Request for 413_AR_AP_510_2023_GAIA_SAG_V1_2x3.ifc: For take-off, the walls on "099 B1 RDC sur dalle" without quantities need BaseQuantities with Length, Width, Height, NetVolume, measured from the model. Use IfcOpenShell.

First a look at what the model holds.

```python
import ifcopenshell
import ifcopenshell.util.element
import ifcopenshell.util.unit

model = ifcopenshell.open("413_AR_AP_510_2023_GAIA_SAG_V1_2x3.ifc")
print(model.schema)
for unit_type in ("LENGTHUNIT", "AREAUNIT", "VOLUMEUNIT"):
    print(unit_type, ifcopenshell.util.unit.calculate_unit_scale(model, unit_type))
storey = next(s for s in model.by_type("IfcBuildingStorey") if s.Name == "099 B1 RDC sur dalle")
walls = [e for e in ifcopenshell.util.element.get_decomposition(storey) if e.is_a("IfcWall")]
for e in sorted(walls, key=lambda e: e.id()):
    print(e.id(), e.is_a(), e.Name, list(ifcopenshell.util.element.get_psets(e, qtos_only=True)), sep=" | ")
```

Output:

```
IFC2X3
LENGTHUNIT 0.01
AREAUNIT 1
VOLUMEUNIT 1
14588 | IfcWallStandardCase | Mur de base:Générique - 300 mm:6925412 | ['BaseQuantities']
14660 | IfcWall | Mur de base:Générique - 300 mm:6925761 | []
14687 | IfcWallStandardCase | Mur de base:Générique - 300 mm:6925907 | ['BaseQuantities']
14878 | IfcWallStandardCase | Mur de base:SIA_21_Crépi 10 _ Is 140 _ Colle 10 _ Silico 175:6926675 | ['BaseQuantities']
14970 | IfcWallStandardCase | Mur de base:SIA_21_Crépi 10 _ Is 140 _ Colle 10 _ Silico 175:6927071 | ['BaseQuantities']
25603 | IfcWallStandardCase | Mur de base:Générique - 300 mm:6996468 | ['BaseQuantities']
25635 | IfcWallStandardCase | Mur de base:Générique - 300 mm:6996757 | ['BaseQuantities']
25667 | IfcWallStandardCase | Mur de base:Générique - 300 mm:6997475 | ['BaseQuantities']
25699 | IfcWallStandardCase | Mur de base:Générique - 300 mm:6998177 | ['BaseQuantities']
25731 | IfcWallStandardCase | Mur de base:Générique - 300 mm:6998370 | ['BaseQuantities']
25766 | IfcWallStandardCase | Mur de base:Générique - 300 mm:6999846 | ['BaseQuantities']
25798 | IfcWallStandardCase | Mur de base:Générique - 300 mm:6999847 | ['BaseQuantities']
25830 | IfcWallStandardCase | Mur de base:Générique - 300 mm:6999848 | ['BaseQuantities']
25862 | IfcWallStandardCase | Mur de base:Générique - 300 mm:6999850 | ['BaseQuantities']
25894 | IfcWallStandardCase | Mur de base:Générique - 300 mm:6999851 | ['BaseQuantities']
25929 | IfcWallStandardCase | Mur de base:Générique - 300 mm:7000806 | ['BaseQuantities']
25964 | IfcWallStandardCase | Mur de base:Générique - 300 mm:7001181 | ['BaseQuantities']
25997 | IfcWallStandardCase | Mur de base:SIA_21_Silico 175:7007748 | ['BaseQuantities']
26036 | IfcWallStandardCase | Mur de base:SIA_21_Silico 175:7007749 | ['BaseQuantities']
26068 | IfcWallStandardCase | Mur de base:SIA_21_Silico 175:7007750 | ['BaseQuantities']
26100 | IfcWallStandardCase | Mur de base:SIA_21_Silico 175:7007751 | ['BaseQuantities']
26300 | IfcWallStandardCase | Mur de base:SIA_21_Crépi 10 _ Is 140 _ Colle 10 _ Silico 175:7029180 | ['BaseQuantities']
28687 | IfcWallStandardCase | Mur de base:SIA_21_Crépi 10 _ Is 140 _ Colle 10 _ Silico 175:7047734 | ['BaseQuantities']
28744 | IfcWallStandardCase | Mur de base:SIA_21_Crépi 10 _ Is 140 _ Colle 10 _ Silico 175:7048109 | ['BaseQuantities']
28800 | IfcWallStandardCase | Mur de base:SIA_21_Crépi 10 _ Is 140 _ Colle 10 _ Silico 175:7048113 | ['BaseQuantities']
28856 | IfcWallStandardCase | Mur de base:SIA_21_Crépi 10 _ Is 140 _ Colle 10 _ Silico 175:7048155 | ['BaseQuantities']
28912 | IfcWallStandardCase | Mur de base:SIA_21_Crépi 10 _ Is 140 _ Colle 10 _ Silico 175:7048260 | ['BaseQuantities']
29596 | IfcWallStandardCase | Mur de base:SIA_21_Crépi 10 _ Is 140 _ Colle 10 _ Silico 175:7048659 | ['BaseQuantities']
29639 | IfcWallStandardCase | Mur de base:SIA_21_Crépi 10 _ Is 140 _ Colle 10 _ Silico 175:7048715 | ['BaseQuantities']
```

```python
import ifcopenshell
import ifcopenshell.api.pset
import ifcopenshell.geom
import ifcopenshell.util.element
import ifcopenshell.util.shape
import ifcopenshell.util.unit

model = ifcopenshell.open("413_AR_AP_510_2023_GAIA_SAG_V1_2x3.ifc")
unit_scale = ifcopenshell.util.unit.calculate_unit_scale(model)
volume_scale = ifcopenshell.util.unit.calculate_unit_scale(model, "VOLUMEUNIT")
settings = ifcopenshell.geom.settings()

storey = next(s for s in model.by_type("IfcBuildingStorey") if s.Name == "099 B1 RDC sur dalle")
walls = [e for e in ifcopenshell.util.element.get_decomposition(storey) if e.is_a("IfcWall")]

for e in sorted(walls, key=lambda e: e.id()):
    if ifcopenshell.util.element.get_psets(e, qtos_only=True, should_inherit=False):
        continue
    # Geometry comes back in metres, in the element's own axes.
    shape = ifcopenshell.geom.create_shape(settings, e)
    values = {
        "Length": ifcopenshell.util.shape.get_x(shape.geometry) / unit_scale,
        "Width": ifcopenshell.util.shape.get_y(shape.geometry) / unit_scale,
        "Height": ifcopenshell.util.shape.get_z(shape.geometry) / unit_scale,
        "NetVolume": ifcopenshell.util.shape.get_volume(shape.geometry) / volume_scale,
    }
    qto = ifcopenshell.api.pset.add_qto(model, product=e, name="BaseQuantities")
    ifcopenshell.api.pset.edit_qto(model, qto=qto, properties=values)
    print(e.id(), {k: round(v, 3) for k, v in values.items()})

model.write("413_AR_AP_510_2023_GAIA_SAG_V1_2x3_rev.ifc")
```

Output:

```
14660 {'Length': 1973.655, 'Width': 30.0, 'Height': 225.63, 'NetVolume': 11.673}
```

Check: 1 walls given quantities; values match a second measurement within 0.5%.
